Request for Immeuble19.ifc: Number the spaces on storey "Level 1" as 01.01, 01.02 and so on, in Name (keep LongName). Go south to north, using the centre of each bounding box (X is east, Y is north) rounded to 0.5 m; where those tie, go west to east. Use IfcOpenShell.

First a look at what the model holds.

```python
import ifcopenshell
import ifcopenshell.util.element
import ifcopenshell.util.placement

model = ifcopenshell.open("Immeuble19.ifc")
print(model.schema)
storey = next(s for s in model.by_type("IfcBuildingStorey") if s.Name == "Level 1")
spaces = [e for e in ifcopenshell.util.element.get_decomposition(storey) if e.is_a("IfcSpace")]
for e in sorted(spaces, key=lambda e: e.id()):
    origin = ifcopenshell.util.placement.get_local_placement(e.ObjectPlacement)[:3, 3]
    print(e.id(), e.Name, e.LongName, origin.round(2) + 0.0, sep=" | ")
```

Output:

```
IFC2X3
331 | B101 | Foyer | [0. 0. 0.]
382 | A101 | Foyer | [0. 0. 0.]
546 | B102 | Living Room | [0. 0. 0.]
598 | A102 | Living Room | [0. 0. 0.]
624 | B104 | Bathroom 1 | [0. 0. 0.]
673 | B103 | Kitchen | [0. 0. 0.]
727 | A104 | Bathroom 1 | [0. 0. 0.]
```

```python
import ifcopenshell
import ifcopenshell.geom
import ifcopenshell.util.element
import ifcopenshell.util.shape

model = ifcopenshell.open("Immeuble19.ifc")
settings = ifcopenshell.geom.settings()
settings.set("use-world-coords", True)


def centre(element):
    shape = ifcopenshell.geom.create_shape(settings, element)
    return ifcopenshell.util.shape.get_bbox_centroid(shape.geometry)


storey = next(s for s in model.by_type("IfcBuildingStorey") if s.Name == "Level 1")
spaces = [e for e in ifcopenshell.util.element.get_decomposition(storey) if e.is_a("IfcSpace")]

# Insertion points can sit at a corner or the storey origin, so sort by the geometry (in metres).
centres = {e: centre(e) for e in spaces}
spaces.sort(key=lambda e: (round(centres[e][1] / 0.5), centres[e][0]))

for i, e in enumerate(spaces, start=1):
    number = f"01.{i:02d}"
    e.Name = number
    print(e.id(), number)

model.write("Immeuble19-out.ifc")
```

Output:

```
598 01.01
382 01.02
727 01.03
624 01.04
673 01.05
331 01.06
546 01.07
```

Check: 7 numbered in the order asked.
